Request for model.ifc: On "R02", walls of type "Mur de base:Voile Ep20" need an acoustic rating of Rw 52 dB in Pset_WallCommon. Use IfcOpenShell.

First a look at what the model holds.

```python
import ifcopenshell
import ifcopenshell.util.element

model = ifcopenshell.open("model.ifc")
print(model.schema)
storey = next(s for s in model.by_type("IfcBuildingStorey") if s.Name == "R02")
walls = [e for e in ifcopenshell.util.element.get_decomposition(storey) if e.is_a("IfcWall")]
seen = {}
for e in walls:
    element_type = ifcopenshell.util.element.get_type(e)
    key = (element_type.Name if element_type != e and element_type else None, ifcopenshell.util.element.get_pset(e, "Pset_WallCommon", "AcousticRating"))
    seen[key] = seen.get(key, 0) + 1
for (name, value), count in sorted(seen.items(), key=str):
    print(count, "x", name, "|", value)
```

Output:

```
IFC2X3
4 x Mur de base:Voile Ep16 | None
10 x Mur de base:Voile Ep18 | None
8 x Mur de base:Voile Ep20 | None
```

```python
import ifcopenshell
import ifcopenshell.api.pset
import ifcopenshell.util.element

model = ifcopenshell.open("model.ifc")

storey = next(s for s in model.by_type("IfcBuildingStorey") if s.Name == "R02")
walls = [e for e in ifcopenshell.util.element.get_decomposition(storey) if e.is_a("IfcWall")]

count = 0
for e in walls:
    element_type = ifcopenshell.util.element.get_type(e)
    if element_type in (None, e) or element_type.Name != "Mur de base:Voile Ep20":
        continue
    # add_pset returns the element's existing set when there is one.
    pset = ifcopenshell.api.pset.add_pset(model, product=e, name="Pset_WallCommon")
    ifcopenshell.api.pset.edit_pset(model, pset=pset, properties={"AcousticRating": "Rw 52 dB"})
    count += 1

print(count, "walls updated")

model.write("model_rev.ifc")
```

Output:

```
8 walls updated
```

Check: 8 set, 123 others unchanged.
